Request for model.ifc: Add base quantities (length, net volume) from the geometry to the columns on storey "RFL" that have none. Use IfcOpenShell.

First a look at what the model holds.

```python
import ifcopenshell
import ifcopenshell.util.element
import ifcopenshell.util.unit

model = ifcopenshell.open("model.ifc")
print(model.schema)
for unit_type in ("LENGTHUNIT", "AREAUNIT", "VOLUMEUNIT"):
    print(unit_type, ifcopenshell.util.unit.calculate_unit_scale(model, unit_type))
storey = next(s for s in model.by_type("IfcBuildingStorey") if s.Name == "RFL")
columns = [e for e in ifcopenshell.util.element.get_decomposition(storey) if e.is_a("IfcColumn")]
for e in sorted(columns, key=lambda e: e.id()):
    print(e.id(), e.is_a(), e.Name, list(ifcopenshell.util.element.get_psets(e, qtos_only=True)), sep=" | ")
```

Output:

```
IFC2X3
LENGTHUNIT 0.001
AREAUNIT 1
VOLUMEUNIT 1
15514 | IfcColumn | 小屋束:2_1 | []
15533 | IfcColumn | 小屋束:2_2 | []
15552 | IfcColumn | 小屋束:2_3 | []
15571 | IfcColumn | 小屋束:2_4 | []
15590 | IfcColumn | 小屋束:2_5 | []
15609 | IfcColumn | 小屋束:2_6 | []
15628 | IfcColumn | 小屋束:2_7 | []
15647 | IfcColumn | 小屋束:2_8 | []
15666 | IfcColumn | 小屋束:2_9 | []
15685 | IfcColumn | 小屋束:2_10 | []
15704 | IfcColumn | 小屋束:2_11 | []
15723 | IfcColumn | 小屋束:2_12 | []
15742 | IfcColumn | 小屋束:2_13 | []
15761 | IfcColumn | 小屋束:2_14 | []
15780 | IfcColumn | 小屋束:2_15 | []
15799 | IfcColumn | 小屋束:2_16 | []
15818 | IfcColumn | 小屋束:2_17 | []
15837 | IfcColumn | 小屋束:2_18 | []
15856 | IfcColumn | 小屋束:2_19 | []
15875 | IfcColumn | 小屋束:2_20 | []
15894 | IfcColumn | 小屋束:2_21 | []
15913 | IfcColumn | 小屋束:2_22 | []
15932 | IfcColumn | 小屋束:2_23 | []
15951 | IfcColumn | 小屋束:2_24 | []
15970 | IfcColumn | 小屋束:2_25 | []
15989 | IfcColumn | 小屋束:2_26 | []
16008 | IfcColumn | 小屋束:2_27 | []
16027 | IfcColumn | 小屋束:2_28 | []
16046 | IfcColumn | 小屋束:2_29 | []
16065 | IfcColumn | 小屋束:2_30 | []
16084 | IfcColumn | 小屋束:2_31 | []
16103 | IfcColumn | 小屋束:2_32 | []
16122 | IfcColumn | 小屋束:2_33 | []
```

```python
import ifcopenshell
import ifcopenshell.api.pset
import ifcopenshell.geom
import ifcopenshell.util.element
import ifcopenshell.util.shape
import ifcopenshell.util.unit

model = ifcopenshell.open("model.ifc")
unit_scale = ifcopenshell.util.unit.calculate_unit_scale(model)
volume_scale = ifcopenshell.util.unit.calculate_unit_scale(model, "VOLUMEUNIT")
settings = ifcopenshell.geom.settings()

storey = next(s for s in model.by_type("IfcBuildingStorey") if s.Name == "RFL")
columns = [e for e in ifcopenshell.util.element.get_decomposition(storey) if e.is_a("IfcColumn")]

for e in sorted(columns, key=lambda e: e.id()):
    if ifcopenshell.util.element.get_psets(e, qtos_only=True, should_inherit=False):
        continue
    # Geometry comes back in metres, in the element's own axes.
    shape = ifcopenshell.geom.create_shape(settings, e)
    values = {
        "Length": ifcopenshell.util.shape.get_z(shape.geometry) / unit_scale,
        "NetVolume": ifcopenshell.util.shape.get_volume(shape.geometry) / volume_scale,
    }
    qto = ifcopenshell.api.pset.add_qto(model, product=e, name="BaseQuantities")
    ifcopenshell.api.pset.edit_qto(model, qto=qto, properties=values)
    print(e.id(), {k: round(v, 3) for k, v in values.items()})

model.write("model_updated.ifc")
```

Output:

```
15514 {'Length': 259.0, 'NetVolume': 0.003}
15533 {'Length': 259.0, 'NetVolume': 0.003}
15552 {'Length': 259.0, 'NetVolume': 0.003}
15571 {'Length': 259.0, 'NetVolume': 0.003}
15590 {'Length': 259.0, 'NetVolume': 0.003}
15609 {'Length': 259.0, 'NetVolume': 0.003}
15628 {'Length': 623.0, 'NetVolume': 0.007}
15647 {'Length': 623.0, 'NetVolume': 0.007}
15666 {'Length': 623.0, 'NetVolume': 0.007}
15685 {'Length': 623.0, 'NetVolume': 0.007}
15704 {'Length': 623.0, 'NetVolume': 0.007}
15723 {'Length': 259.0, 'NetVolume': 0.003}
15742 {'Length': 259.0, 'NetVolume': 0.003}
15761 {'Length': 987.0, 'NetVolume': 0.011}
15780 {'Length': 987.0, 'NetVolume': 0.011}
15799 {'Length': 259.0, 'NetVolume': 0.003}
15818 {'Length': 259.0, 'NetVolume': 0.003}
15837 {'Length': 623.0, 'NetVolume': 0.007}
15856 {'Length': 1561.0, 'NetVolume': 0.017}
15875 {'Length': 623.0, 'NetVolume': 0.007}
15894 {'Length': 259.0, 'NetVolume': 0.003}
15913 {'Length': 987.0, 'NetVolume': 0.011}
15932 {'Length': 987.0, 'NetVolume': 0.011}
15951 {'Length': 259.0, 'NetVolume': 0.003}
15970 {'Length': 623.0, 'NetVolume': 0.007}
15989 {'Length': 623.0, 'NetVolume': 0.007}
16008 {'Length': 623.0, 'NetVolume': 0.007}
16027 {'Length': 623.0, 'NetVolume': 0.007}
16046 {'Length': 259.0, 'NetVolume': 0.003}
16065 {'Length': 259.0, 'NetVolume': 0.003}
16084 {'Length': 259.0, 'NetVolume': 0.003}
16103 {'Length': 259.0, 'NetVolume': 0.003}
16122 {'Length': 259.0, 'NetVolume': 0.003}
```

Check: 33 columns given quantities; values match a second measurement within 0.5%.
